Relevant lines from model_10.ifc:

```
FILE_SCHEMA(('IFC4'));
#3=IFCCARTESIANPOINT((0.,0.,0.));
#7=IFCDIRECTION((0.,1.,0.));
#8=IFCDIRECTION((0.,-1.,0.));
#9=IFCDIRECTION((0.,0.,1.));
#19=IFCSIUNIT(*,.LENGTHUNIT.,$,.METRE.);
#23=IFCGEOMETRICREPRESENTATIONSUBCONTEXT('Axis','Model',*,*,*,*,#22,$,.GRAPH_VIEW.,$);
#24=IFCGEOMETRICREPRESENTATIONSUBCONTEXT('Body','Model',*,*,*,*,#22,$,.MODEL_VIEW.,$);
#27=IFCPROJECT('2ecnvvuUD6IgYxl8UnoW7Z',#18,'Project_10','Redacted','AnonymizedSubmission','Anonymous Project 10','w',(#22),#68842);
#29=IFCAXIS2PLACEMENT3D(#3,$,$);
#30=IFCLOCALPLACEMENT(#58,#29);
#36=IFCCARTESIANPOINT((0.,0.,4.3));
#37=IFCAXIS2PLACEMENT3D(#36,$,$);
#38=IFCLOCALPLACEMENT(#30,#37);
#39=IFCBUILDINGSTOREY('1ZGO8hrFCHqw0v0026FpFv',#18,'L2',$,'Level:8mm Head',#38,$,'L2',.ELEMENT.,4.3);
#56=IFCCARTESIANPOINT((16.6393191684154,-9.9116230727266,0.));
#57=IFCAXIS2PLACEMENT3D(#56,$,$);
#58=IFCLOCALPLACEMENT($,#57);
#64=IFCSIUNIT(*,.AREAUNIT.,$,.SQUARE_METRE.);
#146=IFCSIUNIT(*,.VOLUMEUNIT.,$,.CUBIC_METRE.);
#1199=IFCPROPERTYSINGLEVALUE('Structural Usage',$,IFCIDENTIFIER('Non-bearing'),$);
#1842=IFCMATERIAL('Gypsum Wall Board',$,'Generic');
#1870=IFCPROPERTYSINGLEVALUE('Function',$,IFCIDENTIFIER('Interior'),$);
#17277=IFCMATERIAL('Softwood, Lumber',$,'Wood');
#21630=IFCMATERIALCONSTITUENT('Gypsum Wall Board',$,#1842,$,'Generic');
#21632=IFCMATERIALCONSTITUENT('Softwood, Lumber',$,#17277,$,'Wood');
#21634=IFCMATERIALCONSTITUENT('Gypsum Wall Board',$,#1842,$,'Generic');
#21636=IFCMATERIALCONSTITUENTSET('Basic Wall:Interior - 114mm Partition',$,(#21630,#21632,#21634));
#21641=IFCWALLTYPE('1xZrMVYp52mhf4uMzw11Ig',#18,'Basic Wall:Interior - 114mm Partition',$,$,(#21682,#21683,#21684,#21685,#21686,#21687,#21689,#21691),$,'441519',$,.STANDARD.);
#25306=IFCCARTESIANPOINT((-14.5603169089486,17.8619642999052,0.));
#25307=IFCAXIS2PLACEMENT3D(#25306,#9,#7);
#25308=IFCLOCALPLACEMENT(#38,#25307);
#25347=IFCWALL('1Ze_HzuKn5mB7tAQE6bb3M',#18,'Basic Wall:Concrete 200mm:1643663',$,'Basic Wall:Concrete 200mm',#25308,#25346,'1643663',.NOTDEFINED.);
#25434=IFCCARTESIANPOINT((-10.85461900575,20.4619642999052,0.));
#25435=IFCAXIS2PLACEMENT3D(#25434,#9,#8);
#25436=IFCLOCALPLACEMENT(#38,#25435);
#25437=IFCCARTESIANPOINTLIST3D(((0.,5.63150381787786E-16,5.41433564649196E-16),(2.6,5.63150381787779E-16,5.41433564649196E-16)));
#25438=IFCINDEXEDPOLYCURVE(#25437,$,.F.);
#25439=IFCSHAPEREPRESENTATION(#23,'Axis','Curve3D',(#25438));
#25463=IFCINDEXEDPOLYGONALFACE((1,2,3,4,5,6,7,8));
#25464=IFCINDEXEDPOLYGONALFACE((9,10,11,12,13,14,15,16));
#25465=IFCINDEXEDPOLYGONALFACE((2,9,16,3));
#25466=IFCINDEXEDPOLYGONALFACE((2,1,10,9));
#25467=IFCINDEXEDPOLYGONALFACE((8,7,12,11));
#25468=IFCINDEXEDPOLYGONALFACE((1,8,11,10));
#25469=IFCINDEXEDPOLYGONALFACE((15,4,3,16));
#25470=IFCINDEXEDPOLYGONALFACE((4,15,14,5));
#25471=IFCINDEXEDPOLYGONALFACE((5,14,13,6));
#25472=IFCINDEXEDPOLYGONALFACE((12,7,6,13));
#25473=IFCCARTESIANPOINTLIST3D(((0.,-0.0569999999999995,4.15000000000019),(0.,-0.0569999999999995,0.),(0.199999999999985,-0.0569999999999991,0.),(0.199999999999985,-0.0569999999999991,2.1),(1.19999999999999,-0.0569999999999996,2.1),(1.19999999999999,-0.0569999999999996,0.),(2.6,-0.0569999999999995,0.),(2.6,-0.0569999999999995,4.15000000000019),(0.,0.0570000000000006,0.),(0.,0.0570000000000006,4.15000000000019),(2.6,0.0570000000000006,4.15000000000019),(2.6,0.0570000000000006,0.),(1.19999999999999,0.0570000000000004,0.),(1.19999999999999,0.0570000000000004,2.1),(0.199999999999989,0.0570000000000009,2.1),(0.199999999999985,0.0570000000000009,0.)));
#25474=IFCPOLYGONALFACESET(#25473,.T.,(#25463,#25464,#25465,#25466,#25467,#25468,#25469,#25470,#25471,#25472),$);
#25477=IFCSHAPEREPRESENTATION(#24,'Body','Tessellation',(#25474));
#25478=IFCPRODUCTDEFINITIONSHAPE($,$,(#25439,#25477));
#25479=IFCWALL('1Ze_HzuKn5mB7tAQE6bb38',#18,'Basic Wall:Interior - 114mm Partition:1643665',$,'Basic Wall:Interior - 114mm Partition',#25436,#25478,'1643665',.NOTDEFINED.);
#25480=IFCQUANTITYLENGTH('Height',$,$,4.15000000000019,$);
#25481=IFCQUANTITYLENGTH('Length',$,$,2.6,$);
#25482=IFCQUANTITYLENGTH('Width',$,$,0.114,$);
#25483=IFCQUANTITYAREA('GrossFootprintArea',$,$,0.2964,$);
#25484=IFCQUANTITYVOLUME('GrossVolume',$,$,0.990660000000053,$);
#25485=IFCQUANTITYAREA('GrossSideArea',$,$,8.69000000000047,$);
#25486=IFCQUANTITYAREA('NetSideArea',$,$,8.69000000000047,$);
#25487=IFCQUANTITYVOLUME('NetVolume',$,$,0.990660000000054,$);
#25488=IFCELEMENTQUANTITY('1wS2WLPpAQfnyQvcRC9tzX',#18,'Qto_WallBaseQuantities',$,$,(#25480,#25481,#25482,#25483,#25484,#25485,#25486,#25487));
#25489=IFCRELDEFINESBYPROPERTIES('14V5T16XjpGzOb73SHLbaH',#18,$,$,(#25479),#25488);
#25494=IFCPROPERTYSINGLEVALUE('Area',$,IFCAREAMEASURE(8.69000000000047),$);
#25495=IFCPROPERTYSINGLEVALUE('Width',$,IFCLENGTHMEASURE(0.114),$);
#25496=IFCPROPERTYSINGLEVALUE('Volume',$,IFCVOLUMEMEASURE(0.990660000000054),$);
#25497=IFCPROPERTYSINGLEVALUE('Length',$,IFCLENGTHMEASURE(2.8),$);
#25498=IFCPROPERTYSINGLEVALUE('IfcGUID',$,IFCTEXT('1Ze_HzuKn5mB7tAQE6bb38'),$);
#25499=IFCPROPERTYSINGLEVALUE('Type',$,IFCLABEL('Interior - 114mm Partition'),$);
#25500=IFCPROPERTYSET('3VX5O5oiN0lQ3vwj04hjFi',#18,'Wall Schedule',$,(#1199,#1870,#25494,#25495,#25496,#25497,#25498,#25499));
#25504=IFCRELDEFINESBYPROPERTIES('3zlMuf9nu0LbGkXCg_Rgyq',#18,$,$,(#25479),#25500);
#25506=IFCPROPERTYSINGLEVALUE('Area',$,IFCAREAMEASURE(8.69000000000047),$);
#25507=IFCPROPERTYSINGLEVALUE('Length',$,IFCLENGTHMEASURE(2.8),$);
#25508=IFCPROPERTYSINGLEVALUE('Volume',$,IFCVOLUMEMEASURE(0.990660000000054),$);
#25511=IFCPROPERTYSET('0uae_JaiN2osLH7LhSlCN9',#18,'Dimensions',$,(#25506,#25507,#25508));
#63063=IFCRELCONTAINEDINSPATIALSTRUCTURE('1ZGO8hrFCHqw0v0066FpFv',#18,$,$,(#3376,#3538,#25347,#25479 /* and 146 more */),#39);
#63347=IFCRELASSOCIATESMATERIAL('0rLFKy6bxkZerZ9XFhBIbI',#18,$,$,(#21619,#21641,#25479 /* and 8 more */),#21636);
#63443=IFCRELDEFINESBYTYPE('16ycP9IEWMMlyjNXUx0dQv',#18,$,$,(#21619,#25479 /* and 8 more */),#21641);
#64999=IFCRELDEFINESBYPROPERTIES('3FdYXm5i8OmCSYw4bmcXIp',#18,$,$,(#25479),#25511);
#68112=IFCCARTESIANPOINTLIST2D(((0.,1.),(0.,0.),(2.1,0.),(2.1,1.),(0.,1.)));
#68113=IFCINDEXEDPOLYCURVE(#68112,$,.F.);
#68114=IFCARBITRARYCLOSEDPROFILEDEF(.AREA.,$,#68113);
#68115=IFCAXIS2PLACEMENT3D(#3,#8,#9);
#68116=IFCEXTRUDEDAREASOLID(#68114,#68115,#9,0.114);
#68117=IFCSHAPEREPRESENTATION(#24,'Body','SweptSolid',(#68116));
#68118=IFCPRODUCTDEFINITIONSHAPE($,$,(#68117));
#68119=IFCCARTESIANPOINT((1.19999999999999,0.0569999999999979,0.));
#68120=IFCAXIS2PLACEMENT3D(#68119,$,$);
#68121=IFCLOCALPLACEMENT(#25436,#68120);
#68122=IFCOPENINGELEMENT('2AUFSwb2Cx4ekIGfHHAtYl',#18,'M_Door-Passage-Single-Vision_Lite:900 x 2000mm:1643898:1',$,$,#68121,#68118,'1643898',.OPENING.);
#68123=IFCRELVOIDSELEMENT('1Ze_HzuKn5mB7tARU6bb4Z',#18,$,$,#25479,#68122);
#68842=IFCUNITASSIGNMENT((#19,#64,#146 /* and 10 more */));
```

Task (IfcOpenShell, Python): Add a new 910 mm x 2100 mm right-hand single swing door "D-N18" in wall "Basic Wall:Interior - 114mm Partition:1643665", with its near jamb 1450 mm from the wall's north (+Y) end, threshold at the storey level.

```python
import numpy as np
import ifcopenshell
import ifcopenshell.api.feature
import ifcopenshell.api.geometry
import ifcopenshell.api.pset
import ifcopenshell.api.root
import ifcopenshell.api.spatial
import ifcopenshell.geom
import ifcopenshell.util.element
import ifcopenshell.util.placement
import ifcopenshell.util.representation
import ifcopenshell.util.shape
import ifcopenshell.util.unit

model = ifcopenshell.open("model_10.ifc")
unit_scale = ifcopenshell.util.unit.calculate_unit_scale(model)
area_scale = ifcopenshell.util.unit.calculate_unit_scale(model, "AREAUNIT")
volume_scale = ifcopenshell.util.unit.calculate_unit_scale(model, "VOLUMEUNIT")
settings = ifcopenshell.geom.settings()


def volume(element):
    """Net volume in cubic metres, openings subtracted."""
    shape = ifcopenshell.geom.create_shape(settings, element)
    return ifcopenshell.util.shape.get_volume(shape.geometry)


wall = model.by_guid("1Ze_HzuKn5mB7tAQE6bb38")
storey = ifcopenshell.util.element.get_container(wall, ifc_class="IfcBuildingStorey")
context = ifcopenshell.util.representation.get_context(model, "Model", "Body", "MODEL_VIEW")
before = volume(wall)

width, height, from_end, sill = 0.91, 2.1, 1.45, 0.0  # metres

# The wall runs along its own X axis, and the end named is its -X end.
wall_shape = ifcopenshell.geom.create_shape(settings, wall)
x, y, z = ifcopenshell.util.shape.get_vertices(wall_shape.geometry).T
start = x.min() + from_end
face, thickness = float(y.min()), float(y.max() - y.min())
wall_matrix = ifcopenshell.util.placement.get_local_placement(wall.ObjectPlacement)
level = ifcopenshell.util.placement.get_local_placement(storey.ObjectPlacement)[2, 3]


def in_wall(x, y):
    """Placement at x, y metres in the wall's axes, at sill height."""
    matrix = wall_matrix.copy()
    matrix[:, 3] = wall_matrix @ np.array([x / unit_scale, y / unit_scale, 0.0, 1.0])
    matrix[2, 3] = level + sill / unit_scale
    return matrix


# Opening: a box that overshoots both wall faces by 50 mm.
opening = ifcopenshell.api.root.create_entity(model, ifc_class="IfcOpeningElement", predefined_type="OPENING")
box = ifcopenshell.api.geometry.add_wall_representation(
    model, context=context, length=width, height=height, thickness=thickness + 0.1
)
ifcopenshell.api.geometry.assign_representation(model, product=opening, representation=box)
ifcopenshell.api.geometry.edit_object_placement(model, product=opening, matrix=in_wall(start, face - 0.05), is_si=False)
ifcopenshell.api.feature.add_feature(model, feature=opening, element=wall)

door = ifcopenshell.api.root.create_entity(model, ifc_class="IfcDoor", name="D-N18", predefined_type="DOOR")
door.OverallWidth, door.OverallHeight = width / unit_scale, height / unit_scale
door.OperationType = "SINGLE_SWING_RIGHT"
body = ifcopenshell.api.geometry.add_door_representation(
    model,
    context=context,
    overall_width=door.OverallWidth,
    overall_height=door.OverallHeight,
    operation_type="SINGLE_SWING_RIGHT",
    lining_properties={"LiningDepth": thickness / unit_scale, "ThresholdDepth": thickness / unit_scale},
)
ifcopenshell.api.geometry.assign_representation(model, product=door, representation=body)
ifcopenshell.api.spatial.assign_container(model, products=[door], relating_structure=storey)
ifcopenshell.api.feature.add_filling(model, opening=opening, element=door)

# The lining spans the wall, so the door starts at the wall face.
ifcopenshell.api.geometry.edit_object_placement(model, product=door, matrix=in_wall(start, face), is_si=False)

after = volume(wall)

# Update the wall's stored quantities.
qto = model.by_id(ifcopenshell.util.element.get_pset(wall, "Qto_WallBaseQuantities", should_inherit=False)["id"])
ifcopenshell.api.pset.edit_qto(model, qto=qto, properties={
    "NetSideArea": after / thickness / area_scale,
    "NetVolume": after / volume_scale,
})
pset = model.by_id(ifcopenshell.util.element.get_pset(wall, "Wall Schedule", should_inherit=False)["id"])
ifcopenshell.api.pset.edit_pset(model, pset=pset, properties={
    "Area": model.create_entity("IfcAreaMeasure", after / thickness / area_scale),
    "Volume": model.create_entity("IfcVolumeMeasure", after / volume_scale),
})
pset = model.by_id(ifcopenshell.util.element.get_pset(wall, "Dimensions", should_inherit=False)["id"])
ifcopenshell.api.pset.edit_pset(model, pset=pset, properties={
    "Area": model.create_entity("IfcAreaMeasure", after / thickness / area_scale),
    "Volume": model.create_entity("IfcVolumeMeasure", after / volume_scale),
})

print(f"wall volume {before:.3f} -> {after:.3f} m3")

model.write("model_10_updated.ifc")
```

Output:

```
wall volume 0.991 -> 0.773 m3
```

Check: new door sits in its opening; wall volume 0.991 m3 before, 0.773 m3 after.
